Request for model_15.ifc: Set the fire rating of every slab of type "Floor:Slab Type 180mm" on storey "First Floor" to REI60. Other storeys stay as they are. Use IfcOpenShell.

First a look at what the model holds.

```python
import ifcopenshell
import ifcopenshell.util.element

model = ifcopenshell.open("model_15.ifc")
print(model.schema)
storey = next(s for s in model.by_type("IfcBuildingStorey") if s.Name == "First Floor")
slabs = [e for e in ifcopenshell.util.element.get_decomposition(storey) if e.is_a("IfcSlab")]
seen = {}
for e in slabs:
    element_type = ifcopenshell.util.element.get_type(e)
    key = (element_type.Name if element_type != e and element_type else None, ifcopenshell.util.element.get_pset(e, "Pset_SlabCommon", "FireRating"))
    seen[key] = seen.get(key, 0) + 1
for (name, value), count in sorted(seen.items(), key=str):
    print(count, "x", name, "|", value)
```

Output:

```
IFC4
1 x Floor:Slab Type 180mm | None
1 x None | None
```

```python
import ifcopenshell
import ifcopenshell.api.pset
import ifcopenshell.util.element

model = ifcopenshell.open("model_15.ifc")

storey = next(s for s in model.by_type("IfcBuildingStorey") if s.Name == "First Floor")
slabs = [e for e in ifcopenshell.util.element.get_decomposition(storey) if e.is_a("IfcSlab")]

count = 0
for e in slabs:
    element_type = ifcopenshell.util.element.get_type(e)
    if element_type in (None, e) or element_type.Name != "Floor:Slab Type 180mm":
        continue
    # add_pset returns the element's existing set when there is one.
    pset = ifcopenshell.api.pset.add_pset(model, product=e, name="Pset_SlabCommon")
    ifcopenshell.api.pset.edit_pset(model, pset=pset, properties={"FireRating": "REI60"})
    count += 1

print(count, "slabs updated")

model.write("model_15_rev.ifc")
```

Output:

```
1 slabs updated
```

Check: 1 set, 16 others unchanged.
